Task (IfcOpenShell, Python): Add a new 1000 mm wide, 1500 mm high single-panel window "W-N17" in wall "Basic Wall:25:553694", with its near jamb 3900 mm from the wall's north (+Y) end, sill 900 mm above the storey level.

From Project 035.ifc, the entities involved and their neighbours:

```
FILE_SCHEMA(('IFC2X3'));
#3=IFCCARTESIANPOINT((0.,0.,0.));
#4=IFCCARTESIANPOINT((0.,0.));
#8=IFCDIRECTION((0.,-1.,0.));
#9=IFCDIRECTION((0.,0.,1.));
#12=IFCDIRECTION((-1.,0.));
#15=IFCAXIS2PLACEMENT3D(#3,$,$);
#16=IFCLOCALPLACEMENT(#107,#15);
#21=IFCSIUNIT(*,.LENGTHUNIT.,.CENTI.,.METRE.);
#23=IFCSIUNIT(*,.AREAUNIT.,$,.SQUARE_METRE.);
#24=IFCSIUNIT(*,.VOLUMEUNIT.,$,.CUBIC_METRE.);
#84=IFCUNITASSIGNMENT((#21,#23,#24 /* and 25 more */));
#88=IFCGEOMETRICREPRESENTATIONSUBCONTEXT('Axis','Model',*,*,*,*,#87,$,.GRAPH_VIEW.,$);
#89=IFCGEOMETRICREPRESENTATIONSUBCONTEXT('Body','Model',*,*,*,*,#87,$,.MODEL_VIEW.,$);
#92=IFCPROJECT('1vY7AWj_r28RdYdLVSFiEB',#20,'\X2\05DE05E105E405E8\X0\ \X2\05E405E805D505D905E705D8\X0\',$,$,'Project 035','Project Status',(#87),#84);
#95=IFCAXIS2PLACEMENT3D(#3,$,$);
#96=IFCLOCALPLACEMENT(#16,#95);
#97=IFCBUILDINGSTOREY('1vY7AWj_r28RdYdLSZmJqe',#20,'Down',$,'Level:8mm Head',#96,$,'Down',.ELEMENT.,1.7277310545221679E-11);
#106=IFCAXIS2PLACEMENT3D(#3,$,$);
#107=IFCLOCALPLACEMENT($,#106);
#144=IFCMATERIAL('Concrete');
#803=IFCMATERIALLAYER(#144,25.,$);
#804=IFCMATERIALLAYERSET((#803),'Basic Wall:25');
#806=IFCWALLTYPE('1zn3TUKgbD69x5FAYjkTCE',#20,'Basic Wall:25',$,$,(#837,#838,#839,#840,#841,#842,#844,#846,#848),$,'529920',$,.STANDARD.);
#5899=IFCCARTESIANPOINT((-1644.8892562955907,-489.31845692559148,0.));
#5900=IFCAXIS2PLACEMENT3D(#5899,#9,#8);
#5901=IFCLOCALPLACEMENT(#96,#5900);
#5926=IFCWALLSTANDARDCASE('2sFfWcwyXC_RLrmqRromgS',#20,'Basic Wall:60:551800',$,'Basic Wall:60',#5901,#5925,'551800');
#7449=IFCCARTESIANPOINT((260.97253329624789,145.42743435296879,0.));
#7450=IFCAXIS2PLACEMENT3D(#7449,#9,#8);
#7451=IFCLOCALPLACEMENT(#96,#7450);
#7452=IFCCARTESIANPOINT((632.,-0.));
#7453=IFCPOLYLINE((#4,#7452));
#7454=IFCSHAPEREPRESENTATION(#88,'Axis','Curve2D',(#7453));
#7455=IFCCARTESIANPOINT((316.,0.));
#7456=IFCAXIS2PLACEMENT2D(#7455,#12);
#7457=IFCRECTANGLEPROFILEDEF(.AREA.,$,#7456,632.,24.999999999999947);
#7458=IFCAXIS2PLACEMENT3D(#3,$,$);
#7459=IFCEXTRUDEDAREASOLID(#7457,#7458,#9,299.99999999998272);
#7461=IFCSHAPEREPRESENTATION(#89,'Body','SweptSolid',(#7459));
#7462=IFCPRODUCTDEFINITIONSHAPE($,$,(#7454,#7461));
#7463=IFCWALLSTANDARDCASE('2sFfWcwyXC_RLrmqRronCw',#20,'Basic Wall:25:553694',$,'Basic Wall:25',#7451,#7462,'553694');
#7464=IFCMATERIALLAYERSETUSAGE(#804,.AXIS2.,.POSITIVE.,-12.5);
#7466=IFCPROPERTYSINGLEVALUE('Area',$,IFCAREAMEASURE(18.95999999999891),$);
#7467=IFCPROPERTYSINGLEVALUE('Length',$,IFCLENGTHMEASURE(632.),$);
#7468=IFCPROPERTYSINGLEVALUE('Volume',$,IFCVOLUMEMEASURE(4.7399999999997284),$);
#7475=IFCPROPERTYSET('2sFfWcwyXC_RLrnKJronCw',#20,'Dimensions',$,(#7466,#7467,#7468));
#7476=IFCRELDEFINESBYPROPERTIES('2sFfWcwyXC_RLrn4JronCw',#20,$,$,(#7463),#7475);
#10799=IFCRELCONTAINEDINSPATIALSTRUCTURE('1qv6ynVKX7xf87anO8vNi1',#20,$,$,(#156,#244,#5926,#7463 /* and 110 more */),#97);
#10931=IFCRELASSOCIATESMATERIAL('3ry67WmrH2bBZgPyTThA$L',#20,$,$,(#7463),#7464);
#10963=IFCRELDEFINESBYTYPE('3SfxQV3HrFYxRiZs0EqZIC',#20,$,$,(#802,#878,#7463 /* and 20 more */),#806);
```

```python
import numpy as np
import ifcopenshell
import ifcopenshell.api.feature
import ifcopenshell.api.geometry
import ifcopenshell.api.pset
import ifcopenshell.api.root
import ifcopenshell.api.spatial
import ifcopenshell.api.type
import ifcopenshell.geom
import ifcopenshell.util.element
import ifcopenshell.util.placement
import ifcopenshell.util.representation
import ifcopenshell.util.shape
import ifcopenshell.util.unit

model = ifcopenshell.open("Project 035.ifc")
unit_scale = ifcopenshell.util.unit.calculate_unit_scale(model)
area_scale = ifcopenshell.util.unit.calculate_unit_scale(model, "AREAUNIT")
volume_scale = ifcopenshell.util.unit.calculate_unit_scale(model, "VOLUMEUNIT")
settings = ifcopenshell.geom.settings()


def volume(element):
    """Net volume in cubic metres, openings subtracted."""
    shape = ifcopenshell.geom.create_shape(settings, element)
    return ifcopenshell.util.shape.get_volume(shape.geometry)


wall = model.by_id(7463)
storey = ifcopenshell.util.element.get_container(wall, ifc_class="IfcBuildingStorey")
context = ifcopenshell.util.representation.get_context(model, "Model", "Body", "MODEL_VIEW")
before = volume(wall)

width, height, from_end, sill = 1, 1.5, 3.9, 0.9  # metres

# The wall runs along its own X axis, and the end named is its -X end.
wall_shape = ifcopenshell.geom.create_shape(settings, wall)
x, y, z = ifcopenshell.util.shape.get_vertices(wall_shape.geometry).T
start = x.min() + from_end
face, thickness = float(y.min()), float(y.max() - y.min())
wall_matrix = ifcopenshell.util.placement.get_local_placement(wall.ObjectPlacement)
level = ifcopenshell.util.placement.get_local_placement(storey.ObjectPlacement)[2, 3]


def in_wall(x, y):
    """Placement at x, y metres in the wall's axes, at sill height."""
    matrix = wall_matrix.copy()
    matrix[:, 3] = wall_matrix @ np.array([x / unit_scale, y / unit_scale, 0.0, 1.0])
    matrix[2, 3] = level + sill / unit_scale
    return matrix


# Opening: a box that overshoots both wall faces by 50 mm.
opening = ifcopenshell.api.root.create_entity(model, ifc_class="IfcOpeningElement")
box = ifcopenshell.api.geometry.add_wall_representation(
    model, context=context, length=width, height=height, thickness=thickness + 0.1
)
ifcopenshell.api.geometry.assign_representation(model, product=opening, representation=box)
ifcopenshell.api.geometry.edit_object_placement(model, product=opening, matrix=in_wall(start, face - 0.05), is_si=False)
ifcopenshell.api.feature.add_feature(model, feature=opening, element=wall)

window = ifcopenshell.api.root.create_entity(model, ifc_class="IfcWindow", name="W-N17")
window.OverallWidth, window.OverallHeight = width / unit_scale, height / unit_scale
body = ifcopenshell.api.geometry.add_window_representation(
    model,
    context=context,
    overall_width=window.OverallWidth,
    overall_height=window.OverallHeight,
    partition_type="SINGLE_PANEL",
)
ifcopenshell.api.geometry.assign_representation(model, product=window, representation=body)
ifcopenshell.api.spatial.assign_container(model, products=[window], relating_structure=storey)
fills = ifcopenshell.api.feature.add_filling(model, opening=opening, element=window)
fills.OwnerHistory = window.OwnerHistory  # required in IFC2X3

# IFC2X3 keeps the operation on the window style.
style = ifcopenshell.api.root.create_entity(model, ifc_class="IfcWindowStyle", name="W-N17")
style.OperationType, style.ConstructionType = "SINGLE_PANEL", "NOTDEFINED"
style.ParameterTakesPrecedence = style.Sizeable = False
ifcopenshell.api.type.assign_type(model, related_objects=[window], relating_type=style)

# Centre the window in the wall's thickness.
ifcopenshell.api.geometry.edit_object_placement(model, product=window, matrix=in_wall(start, face), is_si=False)
window_shape = ifcopenshell.geom.create_shape(settings, window)
depth = ifcopenshell.util.shape.get_vertices(window_shape.geometry)[:, 1]
offset = face + thickness / 2 - (depth.min() + depth.max()) / 2
ifcopenshell.api.geometry.edit_object_placement(model, product=window, matrix=in_wall(start, offset), is_si=False)

after = volume(wall)

# Update the wall's stored quantities.
pset = model.by_id(ifcopenshell.util.element.get_pset(wall, "Dimensions", should_inherit=False)["id"])
ifcopenshell.api.pset.edit_pset(model, pset=pset, properties={
    "Area": model.create_entity("IfcAreaMeasure", after / thickness / area_scale),
    "Volume": model.create_entity("IfcVolumeMeasure", after / volume_scale),
})

print(f"wall volume {before:.3f} -> {after:.3f} m3")

model.write("Project 035_updated.ifc")
```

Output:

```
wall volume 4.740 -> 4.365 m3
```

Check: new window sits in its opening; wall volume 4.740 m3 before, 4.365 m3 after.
